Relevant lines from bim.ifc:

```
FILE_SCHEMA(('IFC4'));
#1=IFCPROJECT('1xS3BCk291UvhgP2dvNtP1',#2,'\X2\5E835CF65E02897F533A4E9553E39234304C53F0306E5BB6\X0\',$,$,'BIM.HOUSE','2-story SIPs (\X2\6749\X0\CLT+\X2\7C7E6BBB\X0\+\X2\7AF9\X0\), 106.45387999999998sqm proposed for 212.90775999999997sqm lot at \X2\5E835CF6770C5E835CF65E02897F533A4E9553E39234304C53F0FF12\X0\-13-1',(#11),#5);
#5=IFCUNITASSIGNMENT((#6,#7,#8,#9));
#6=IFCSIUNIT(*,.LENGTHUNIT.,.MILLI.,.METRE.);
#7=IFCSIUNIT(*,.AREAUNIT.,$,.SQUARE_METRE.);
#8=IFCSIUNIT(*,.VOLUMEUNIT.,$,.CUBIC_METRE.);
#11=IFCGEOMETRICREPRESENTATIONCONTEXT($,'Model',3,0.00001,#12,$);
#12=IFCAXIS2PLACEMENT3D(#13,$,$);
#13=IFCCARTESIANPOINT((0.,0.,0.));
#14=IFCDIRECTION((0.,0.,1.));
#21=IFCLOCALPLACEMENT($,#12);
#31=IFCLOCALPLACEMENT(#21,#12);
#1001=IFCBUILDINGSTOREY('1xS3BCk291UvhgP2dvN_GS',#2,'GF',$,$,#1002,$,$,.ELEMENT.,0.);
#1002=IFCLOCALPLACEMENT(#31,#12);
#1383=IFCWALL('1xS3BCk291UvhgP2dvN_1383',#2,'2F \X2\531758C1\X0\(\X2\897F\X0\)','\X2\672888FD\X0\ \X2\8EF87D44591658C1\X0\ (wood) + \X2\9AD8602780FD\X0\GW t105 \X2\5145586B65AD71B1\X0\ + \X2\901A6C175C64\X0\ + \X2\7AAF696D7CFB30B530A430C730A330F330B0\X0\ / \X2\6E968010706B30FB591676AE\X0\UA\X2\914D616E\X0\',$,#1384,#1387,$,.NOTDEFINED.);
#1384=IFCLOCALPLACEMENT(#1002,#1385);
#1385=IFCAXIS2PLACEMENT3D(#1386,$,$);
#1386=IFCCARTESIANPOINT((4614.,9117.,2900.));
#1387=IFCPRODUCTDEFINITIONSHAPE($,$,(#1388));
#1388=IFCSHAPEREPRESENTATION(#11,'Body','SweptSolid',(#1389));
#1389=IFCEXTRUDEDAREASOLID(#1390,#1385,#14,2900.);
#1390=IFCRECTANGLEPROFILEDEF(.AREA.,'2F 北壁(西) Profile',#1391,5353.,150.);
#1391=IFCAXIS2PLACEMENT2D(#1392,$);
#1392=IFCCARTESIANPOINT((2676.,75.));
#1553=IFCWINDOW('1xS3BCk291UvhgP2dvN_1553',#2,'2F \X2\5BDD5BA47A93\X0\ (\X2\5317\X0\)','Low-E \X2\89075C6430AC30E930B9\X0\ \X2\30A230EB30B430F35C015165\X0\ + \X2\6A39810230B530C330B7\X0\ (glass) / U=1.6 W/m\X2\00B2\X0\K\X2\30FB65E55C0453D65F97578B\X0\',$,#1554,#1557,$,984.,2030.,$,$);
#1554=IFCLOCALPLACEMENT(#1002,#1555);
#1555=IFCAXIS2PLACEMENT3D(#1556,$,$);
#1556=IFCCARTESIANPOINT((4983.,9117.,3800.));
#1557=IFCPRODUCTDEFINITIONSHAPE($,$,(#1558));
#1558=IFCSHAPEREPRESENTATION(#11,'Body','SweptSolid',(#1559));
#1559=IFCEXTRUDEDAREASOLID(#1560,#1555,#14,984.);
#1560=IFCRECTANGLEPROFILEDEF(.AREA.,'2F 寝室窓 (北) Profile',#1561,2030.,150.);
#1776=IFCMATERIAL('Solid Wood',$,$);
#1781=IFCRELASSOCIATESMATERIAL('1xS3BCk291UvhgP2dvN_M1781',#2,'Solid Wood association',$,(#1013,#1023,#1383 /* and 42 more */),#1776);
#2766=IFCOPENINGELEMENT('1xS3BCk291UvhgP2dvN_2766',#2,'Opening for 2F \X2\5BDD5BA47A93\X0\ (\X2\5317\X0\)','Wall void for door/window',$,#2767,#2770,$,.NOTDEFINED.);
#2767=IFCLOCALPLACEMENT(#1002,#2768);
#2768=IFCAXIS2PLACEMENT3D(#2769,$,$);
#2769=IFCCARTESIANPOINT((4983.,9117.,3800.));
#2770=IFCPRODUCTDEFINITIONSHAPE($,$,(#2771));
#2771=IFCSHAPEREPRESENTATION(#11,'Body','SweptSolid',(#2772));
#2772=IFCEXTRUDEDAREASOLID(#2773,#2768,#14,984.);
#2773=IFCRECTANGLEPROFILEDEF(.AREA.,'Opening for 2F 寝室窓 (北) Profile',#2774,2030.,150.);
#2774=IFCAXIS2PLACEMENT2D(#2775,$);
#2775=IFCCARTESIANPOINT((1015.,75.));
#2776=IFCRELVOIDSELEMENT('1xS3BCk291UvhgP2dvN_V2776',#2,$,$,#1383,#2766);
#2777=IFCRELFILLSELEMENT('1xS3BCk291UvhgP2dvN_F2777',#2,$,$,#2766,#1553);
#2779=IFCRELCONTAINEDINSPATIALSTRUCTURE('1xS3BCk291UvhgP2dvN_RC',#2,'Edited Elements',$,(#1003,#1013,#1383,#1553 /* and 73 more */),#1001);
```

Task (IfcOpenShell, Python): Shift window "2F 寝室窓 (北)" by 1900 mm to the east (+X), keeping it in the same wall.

```python
import ifcopenshell
import ifcopenshell.api.geometry
import ifcopenshell.util.placement
import ifcopenshell.util.unit

model = ifcopenshell.open("bim.ifc")
unit_scale = ifcopenshell.util.unit.calculate_unit_scale(model)

window = model.by_guid("1xS3BCk291UvhgP2dvN_1553")
opening = window.FillsVoids[0].RelatingOpeningElement
wall = opening.VoidsElements[0].RelatingBuildingElement

wall_matrix = ifcopenshell.util.placement.get_local_placement(wall.ObjectPlacement)
shift = wall_matrix[:3, 0] * 1.9 / unit_scale
before = ifcopenshell.util.placement.get_local_placement(window.ObjectPlacement)[:3, 3].copy()

# The window is not placed relative to its opening, so move both.
for product in (opening, window):
    matrix = ifcopenshell.util.placement.get_local_placement(product.ObjectPlacement)
    matrix[:3, 3] += shift
    ifcopenshell.api.geometry.edit_object_placement(model, product=product, matrix=matrix, is_si=False)

after = ifcopenshell.util.placement.get_local_placement(window.ObjectPlacement)[:3, 3]
print("window moved by", (after - before).round(3) + 0.0)

model.write("bim_updated.ifc")
```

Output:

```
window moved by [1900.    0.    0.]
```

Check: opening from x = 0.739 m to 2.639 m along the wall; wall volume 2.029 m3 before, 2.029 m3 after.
